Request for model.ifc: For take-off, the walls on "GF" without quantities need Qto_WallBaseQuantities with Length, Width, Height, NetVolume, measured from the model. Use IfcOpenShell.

First a look at what the model holds.

```python
import ifcopenshell
import ifcopenshell.util.element
import ifcopenshell.util.unit

model = ifcopenshell.open("model.ifc")
print(model.schema)
for unit_type in ("LENGTHUNIT", "AREAUNIT", "VOLUMEUNIT"):
    print(unit_type, ifcopenshell.util.unit.calculate_unit_scale(model, unit_type))
storey = next(s for s in model.by_type("IfcBuildingStorey") if s.Name == "GF")
walls = [e for e in ifcopenshell.util.element.get_decomposition(storey) if e.is_a("IfcWall")]
for e in sorted(walls, key=lambda e: e.id()):
    print(e.id(), e.is_a(), e.Name, list(ifcopenshell.util.element.get_psets(e, qtos_only=True)), sep=" | ")
```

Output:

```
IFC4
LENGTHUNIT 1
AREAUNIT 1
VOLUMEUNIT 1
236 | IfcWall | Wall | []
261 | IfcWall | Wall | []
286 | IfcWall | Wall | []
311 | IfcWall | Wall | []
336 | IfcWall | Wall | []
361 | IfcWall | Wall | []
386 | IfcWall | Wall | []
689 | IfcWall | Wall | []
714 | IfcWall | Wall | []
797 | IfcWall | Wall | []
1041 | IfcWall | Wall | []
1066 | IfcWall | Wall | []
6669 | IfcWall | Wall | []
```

```python
import ifcopenshell
import ifcopenshell.api.pset
import ifcopenshell.geom
import ifcopenshell.util.element
import ifcopenshell.util.shape
import ifcopenshell.util.unit

model = ifcopenshell.open("model.ifc")
unit_scale = ifcopenshell.util.unit.calculate_unit_scale(model)
volume_scale = ifcopenshell.util.unit.calculate_unit_scale(model, "VOLUMEUNIT")
settings = ifcopenshell.geom.settings()

storey = next(s for s in model.by_type("IfcBuildingStorey") if s.Name == "GF")
walls = [e for e in ifcopenshell.util.element.get_decomposition(storey) if e.is_a("IfcWall")]

for e in sorted(walls, key=lambda e: e.id()):
    if ifcopenshell.util.element.get_psets(e, qtos_only=True, should_inherit=False):
        continue
    # Geometry comes back in metres, in the element's own axes.
    shape = ifcopenshell.geom.create_shape(settings, e)
    values = {
        "Length": ifcopenshell.util.shape.get_x(shape.geometry) / unit_scale,
        "Width": ifcopenshell.util.shape.get_y(shape.geometry) / unit_scale,
        "Height": ifcopenshell.util.shape.get_z(shape.geometry) / unit_scale,
        "NetVolume": ifcopenshell.util.shape.get_volume(shape.geometry) / volume_scale,
    }
    qto = ifcopenshell.api.pset.add_qto(model, product=e, name="Qto_WallBaseQuantities")
    ifcopenshell.api.pset.edit_qto(model, qto=qto, properties=values)
    print(e.id(), {k: round(v, 3) for k, v in values.items()})

model.write("model-out.ifc")
```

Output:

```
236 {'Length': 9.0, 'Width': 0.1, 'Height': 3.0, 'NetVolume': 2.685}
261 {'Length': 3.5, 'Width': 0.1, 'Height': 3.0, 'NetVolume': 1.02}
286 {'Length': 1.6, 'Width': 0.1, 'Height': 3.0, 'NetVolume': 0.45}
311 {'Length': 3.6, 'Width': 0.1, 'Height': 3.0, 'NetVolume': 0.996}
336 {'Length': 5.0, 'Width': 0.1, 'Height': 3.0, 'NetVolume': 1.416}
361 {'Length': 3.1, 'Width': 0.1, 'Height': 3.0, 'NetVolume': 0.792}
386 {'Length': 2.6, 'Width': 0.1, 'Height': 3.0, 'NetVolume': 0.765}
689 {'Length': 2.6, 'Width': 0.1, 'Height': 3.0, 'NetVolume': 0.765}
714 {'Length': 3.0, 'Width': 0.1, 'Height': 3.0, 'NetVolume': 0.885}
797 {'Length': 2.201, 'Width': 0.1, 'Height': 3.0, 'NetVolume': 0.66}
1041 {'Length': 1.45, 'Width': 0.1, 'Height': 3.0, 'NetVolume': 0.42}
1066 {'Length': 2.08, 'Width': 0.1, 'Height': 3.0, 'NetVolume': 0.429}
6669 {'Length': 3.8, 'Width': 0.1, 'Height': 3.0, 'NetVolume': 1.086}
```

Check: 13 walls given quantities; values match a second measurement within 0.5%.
